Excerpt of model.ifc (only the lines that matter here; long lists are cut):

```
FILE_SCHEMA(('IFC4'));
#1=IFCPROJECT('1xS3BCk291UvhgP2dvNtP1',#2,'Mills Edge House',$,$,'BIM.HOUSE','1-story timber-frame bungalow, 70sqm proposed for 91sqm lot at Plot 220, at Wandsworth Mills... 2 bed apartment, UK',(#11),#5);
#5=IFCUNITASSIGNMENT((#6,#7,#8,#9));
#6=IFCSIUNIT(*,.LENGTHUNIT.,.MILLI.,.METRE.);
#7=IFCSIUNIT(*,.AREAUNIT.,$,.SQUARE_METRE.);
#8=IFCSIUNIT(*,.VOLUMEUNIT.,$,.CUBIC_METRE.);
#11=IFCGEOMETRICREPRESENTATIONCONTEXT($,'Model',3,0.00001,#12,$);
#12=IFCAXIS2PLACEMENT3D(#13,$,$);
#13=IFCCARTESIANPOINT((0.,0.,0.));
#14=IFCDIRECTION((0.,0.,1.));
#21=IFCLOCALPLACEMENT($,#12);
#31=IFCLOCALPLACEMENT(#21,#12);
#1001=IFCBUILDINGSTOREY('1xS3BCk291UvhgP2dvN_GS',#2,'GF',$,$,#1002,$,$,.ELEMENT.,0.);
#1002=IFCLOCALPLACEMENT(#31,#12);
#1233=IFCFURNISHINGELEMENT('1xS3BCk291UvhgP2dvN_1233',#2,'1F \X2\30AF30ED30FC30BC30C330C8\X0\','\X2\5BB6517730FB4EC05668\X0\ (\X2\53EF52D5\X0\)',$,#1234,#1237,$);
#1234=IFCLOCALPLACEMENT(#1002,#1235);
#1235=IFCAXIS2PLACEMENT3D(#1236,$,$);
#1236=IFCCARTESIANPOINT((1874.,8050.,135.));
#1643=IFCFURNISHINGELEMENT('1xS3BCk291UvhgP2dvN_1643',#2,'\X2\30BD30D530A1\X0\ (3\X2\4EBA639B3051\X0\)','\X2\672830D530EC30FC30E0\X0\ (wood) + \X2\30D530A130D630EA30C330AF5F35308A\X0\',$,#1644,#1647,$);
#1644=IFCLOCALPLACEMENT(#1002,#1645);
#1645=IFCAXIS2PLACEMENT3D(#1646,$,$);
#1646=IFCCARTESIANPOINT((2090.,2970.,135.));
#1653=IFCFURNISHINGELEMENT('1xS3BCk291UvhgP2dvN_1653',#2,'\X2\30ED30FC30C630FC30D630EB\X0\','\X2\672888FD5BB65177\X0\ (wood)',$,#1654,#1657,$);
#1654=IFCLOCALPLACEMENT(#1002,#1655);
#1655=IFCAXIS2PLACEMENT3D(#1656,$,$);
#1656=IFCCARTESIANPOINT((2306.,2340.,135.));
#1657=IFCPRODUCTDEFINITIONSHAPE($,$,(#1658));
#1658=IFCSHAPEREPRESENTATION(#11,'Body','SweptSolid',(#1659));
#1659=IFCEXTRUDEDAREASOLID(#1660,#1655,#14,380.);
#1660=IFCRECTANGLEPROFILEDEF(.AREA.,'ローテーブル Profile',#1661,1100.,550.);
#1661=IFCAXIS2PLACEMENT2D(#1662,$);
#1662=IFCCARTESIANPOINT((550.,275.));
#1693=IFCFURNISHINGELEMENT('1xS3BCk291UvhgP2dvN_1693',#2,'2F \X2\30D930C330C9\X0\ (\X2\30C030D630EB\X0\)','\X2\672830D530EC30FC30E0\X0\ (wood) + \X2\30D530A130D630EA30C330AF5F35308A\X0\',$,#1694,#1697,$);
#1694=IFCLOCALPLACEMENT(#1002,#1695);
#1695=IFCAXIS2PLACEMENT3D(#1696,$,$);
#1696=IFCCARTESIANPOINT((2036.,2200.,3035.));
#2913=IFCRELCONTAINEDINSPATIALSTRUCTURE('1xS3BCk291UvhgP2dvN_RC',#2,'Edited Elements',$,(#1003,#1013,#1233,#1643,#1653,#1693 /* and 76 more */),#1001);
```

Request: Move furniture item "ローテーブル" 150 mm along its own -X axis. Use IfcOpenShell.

```python
import ifcopenshell
import ifcopenshell.api.geometry
import ifcopenshell.util.placement
import ifcopenshell.util.unit

model = ifcopenshell.open("model.ifc")
unit_scale = ifcopenshell.util.unit.calculate_unit_scale(model)

item = model.by_id(1653)
matrix = ifcopenshell.util.placement.get_local_placement(item.ObjectPlacement)
matrix[:3, 3] -= matrix[:3, 0] * 0.15 / unit_scale
ifcopenshell.api.geometry.edit_object_placement(model, product=item, matrix=matrix, is_si=False)

print(ifcopenshell.util.placement.get_local_placement(item.ObjectPlacement).round(3) + 0.0)

model.write("model-out.ifc")
```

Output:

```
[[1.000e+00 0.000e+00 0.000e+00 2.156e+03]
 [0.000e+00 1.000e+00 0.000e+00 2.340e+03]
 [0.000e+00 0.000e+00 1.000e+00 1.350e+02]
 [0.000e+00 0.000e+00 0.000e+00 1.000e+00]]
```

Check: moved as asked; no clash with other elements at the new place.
